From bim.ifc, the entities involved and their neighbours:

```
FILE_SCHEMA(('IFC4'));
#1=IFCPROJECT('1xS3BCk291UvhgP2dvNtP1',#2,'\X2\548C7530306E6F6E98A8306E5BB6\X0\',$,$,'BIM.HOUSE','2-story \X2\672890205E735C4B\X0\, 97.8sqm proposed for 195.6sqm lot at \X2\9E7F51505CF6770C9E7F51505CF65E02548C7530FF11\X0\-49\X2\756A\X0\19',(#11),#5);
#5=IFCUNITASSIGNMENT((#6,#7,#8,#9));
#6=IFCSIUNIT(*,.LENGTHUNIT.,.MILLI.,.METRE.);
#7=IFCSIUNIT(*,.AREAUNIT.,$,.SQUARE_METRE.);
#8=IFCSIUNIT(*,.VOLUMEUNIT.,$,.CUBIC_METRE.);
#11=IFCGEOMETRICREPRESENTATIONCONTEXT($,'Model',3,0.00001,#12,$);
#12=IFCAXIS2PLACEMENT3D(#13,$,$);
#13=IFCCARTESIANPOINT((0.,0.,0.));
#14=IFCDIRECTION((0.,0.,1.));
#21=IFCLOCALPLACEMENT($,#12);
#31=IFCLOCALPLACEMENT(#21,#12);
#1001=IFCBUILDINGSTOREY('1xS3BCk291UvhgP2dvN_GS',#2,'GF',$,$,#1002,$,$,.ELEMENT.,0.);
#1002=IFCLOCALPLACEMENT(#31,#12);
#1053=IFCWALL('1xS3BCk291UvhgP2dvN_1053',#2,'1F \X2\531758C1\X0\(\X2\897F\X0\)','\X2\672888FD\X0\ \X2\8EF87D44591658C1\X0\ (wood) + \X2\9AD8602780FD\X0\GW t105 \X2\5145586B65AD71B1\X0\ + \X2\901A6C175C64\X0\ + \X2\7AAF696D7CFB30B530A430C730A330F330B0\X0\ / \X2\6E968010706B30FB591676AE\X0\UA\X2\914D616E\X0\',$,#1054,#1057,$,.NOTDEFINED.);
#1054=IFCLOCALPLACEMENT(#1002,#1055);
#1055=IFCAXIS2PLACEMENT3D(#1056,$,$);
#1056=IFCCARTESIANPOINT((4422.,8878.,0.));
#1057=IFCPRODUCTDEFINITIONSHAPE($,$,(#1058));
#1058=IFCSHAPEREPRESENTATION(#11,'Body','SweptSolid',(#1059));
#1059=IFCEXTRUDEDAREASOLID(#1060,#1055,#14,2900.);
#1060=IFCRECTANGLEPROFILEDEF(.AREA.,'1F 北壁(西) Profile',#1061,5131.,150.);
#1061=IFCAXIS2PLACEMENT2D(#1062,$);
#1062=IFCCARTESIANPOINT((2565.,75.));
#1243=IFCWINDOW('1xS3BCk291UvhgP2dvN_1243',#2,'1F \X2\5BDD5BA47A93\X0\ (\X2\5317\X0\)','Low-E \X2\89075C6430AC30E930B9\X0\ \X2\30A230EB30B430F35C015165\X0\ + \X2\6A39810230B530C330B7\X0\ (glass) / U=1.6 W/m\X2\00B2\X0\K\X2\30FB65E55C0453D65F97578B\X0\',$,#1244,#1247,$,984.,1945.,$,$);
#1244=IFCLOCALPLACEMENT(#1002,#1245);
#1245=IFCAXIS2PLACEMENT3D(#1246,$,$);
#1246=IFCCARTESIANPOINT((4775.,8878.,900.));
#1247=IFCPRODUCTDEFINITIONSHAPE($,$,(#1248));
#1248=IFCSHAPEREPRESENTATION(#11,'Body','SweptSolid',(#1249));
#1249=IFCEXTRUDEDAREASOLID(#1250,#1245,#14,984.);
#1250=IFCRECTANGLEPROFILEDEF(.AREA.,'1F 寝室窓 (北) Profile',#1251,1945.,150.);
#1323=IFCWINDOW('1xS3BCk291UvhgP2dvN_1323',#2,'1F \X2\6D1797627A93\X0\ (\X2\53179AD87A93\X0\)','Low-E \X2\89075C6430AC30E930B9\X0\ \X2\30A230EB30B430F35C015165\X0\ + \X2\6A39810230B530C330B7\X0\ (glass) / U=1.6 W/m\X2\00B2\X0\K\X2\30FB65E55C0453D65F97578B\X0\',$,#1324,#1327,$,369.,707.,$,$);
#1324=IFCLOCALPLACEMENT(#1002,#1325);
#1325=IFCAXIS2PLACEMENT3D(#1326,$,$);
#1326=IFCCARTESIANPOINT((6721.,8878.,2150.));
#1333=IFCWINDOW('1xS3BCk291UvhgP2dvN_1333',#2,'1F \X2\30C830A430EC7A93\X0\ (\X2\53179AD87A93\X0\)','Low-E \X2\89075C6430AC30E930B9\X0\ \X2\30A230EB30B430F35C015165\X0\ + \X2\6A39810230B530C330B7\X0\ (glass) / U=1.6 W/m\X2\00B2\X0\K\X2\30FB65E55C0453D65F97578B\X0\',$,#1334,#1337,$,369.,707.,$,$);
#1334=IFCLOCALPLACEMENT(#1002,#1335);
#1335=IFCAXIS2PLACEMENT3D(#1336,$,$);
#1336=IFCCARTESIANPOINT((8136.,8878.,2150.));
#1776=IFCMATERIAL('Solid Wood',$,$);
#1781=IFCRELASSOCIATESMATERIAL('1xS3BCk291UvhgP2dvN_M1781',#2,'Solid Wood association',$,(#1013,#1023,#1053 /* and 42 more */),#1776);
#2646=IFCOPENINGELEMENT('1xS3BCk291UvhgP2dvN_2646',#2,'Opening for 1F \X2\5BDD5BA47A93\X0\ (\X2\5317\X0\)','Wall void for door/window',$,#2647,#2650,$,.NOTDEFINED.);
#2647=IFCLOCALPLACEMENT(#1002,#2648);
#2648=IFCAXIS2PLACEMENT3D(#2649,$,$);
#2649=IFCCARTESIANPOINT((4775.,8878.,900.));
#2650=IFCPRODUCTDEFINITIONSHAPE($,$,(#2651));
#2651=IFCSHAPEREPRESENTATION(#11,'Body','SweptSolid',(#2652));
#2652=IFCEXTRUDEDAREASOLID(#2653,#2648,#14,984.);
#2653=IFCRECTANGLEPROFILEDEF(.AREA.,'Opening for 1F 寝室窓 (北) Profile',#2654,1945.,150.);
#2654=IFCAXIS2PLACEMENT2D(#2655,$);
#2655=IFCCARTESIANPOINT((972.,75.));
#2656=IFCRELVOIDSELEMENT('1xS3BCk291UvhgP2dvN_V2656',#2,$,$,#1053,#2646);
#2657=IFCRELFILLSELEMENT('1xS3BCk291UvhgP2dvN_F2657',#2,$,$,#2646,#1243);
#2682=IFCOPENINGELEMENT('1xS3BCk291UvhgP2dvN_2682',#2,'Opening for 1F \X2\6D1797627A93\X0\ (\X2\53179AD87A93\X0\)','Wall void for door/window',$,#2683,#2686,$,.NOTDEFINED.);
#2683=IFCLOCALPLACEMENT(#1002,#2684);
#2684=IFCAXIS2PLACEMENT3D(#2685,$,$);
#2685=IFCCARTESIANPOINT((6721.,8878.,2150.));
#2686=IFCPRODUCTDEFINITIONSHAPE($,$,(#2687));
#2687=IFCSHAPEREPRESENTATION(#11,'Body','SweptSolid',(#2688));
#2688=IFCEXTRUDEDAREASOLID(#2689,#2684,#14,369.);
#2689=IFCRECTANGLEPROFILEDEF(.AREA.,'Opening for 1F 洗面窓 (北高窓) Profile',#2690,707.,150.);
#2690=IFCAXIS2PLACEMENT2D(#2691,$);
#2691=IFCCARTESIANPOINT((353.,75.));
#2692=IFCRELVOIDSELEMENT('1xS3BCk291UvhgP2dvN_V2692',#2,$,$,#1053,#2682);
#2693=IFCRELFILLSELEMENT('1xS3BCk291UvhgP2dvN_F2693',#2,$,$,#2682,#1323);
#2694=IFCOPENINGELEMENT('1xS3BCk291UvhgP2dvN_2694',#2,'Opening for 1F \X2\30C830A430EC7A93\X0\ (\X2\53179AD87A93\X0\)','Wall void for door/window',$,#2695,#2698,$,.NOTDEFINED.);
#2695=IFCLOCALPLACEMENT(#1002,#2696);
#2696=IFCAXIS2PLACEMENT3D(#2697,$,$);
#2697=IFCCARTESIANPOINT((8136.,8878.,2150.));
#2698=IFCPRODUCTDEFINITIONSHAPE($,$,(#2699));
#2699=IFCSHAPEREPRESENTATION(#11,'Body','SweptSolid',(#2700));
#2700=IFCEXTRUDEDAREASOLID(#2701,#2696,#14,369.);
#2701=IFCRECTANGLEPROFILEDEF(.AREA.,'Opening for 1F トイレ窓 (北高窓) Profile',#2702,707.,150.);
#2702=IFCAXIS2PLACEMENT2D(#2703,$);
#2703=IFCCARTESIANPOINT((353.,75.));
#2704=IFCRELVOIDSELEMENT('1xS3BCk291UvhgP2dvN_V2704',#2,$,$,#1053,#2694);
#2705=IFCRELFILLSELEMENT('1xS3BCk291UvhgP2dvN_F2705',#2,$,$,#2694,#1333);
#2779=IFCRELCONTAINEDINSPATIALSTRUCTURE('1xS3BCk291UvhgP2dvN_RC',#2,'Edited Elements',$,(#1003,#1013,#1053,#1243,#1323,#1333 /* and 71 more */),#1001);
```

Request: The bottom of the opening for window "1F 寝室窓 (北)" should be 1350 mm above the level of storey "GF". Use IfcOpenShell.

```python
import numpy as np
import ifcopenshell
import ifcopenshell.api.geometry
import ifcopenshell.geom
import ifcopenshell.util.element
import ifcopenshell.util.placement
import ifcopenshell.util.shape
import ifcopenshell.util.unit

model = ifcopenshell.open("bim.ifc")
unit_scale = ifcopenshell.util.unit.calculate_unit_scale(model)

window = model.by_id(1243)
opening = window.FillsVoids[0].RelatingOpeningElement
storey = ifcopenshell.util.element.get_container(window, ifc_class="IfcBuildingStorey")
level = ifcopenshell.util.placement.get_local_placement(storey.ObjectPlacement)[2, 3]

# The opening's origin need not be at the sill, so measure its lowest point.
shape = ifcopenshell.geom.create_shape(ifcopenshell.geom.settings(), opening)
bottom = ifcopenshell.util.shape.get_shape_bottom_elevation(shape, shape.geometry) / unit_scale
dz = level + 1350.0 - bottom

shift = np.array([0.0, 0.0, dz])
# The window is not placed relative to its opening, so move both.
for product in (opening, window):
    matrix = ifcopenshell.util.placement.get_local_placement(product.ObjectPlacement)
    matrix[:3, 3] += shift
    ifcopenshell.api.geometry.edit_object_placement(model, product=product, matrix=matrix, is_si=False)

print(f"moved by {dz * unit_scale:+.3f} m")

model.write("bim_updated.ifc")
```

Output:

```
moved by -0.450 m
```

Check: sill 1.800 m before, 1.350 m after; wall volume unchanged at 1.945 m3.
